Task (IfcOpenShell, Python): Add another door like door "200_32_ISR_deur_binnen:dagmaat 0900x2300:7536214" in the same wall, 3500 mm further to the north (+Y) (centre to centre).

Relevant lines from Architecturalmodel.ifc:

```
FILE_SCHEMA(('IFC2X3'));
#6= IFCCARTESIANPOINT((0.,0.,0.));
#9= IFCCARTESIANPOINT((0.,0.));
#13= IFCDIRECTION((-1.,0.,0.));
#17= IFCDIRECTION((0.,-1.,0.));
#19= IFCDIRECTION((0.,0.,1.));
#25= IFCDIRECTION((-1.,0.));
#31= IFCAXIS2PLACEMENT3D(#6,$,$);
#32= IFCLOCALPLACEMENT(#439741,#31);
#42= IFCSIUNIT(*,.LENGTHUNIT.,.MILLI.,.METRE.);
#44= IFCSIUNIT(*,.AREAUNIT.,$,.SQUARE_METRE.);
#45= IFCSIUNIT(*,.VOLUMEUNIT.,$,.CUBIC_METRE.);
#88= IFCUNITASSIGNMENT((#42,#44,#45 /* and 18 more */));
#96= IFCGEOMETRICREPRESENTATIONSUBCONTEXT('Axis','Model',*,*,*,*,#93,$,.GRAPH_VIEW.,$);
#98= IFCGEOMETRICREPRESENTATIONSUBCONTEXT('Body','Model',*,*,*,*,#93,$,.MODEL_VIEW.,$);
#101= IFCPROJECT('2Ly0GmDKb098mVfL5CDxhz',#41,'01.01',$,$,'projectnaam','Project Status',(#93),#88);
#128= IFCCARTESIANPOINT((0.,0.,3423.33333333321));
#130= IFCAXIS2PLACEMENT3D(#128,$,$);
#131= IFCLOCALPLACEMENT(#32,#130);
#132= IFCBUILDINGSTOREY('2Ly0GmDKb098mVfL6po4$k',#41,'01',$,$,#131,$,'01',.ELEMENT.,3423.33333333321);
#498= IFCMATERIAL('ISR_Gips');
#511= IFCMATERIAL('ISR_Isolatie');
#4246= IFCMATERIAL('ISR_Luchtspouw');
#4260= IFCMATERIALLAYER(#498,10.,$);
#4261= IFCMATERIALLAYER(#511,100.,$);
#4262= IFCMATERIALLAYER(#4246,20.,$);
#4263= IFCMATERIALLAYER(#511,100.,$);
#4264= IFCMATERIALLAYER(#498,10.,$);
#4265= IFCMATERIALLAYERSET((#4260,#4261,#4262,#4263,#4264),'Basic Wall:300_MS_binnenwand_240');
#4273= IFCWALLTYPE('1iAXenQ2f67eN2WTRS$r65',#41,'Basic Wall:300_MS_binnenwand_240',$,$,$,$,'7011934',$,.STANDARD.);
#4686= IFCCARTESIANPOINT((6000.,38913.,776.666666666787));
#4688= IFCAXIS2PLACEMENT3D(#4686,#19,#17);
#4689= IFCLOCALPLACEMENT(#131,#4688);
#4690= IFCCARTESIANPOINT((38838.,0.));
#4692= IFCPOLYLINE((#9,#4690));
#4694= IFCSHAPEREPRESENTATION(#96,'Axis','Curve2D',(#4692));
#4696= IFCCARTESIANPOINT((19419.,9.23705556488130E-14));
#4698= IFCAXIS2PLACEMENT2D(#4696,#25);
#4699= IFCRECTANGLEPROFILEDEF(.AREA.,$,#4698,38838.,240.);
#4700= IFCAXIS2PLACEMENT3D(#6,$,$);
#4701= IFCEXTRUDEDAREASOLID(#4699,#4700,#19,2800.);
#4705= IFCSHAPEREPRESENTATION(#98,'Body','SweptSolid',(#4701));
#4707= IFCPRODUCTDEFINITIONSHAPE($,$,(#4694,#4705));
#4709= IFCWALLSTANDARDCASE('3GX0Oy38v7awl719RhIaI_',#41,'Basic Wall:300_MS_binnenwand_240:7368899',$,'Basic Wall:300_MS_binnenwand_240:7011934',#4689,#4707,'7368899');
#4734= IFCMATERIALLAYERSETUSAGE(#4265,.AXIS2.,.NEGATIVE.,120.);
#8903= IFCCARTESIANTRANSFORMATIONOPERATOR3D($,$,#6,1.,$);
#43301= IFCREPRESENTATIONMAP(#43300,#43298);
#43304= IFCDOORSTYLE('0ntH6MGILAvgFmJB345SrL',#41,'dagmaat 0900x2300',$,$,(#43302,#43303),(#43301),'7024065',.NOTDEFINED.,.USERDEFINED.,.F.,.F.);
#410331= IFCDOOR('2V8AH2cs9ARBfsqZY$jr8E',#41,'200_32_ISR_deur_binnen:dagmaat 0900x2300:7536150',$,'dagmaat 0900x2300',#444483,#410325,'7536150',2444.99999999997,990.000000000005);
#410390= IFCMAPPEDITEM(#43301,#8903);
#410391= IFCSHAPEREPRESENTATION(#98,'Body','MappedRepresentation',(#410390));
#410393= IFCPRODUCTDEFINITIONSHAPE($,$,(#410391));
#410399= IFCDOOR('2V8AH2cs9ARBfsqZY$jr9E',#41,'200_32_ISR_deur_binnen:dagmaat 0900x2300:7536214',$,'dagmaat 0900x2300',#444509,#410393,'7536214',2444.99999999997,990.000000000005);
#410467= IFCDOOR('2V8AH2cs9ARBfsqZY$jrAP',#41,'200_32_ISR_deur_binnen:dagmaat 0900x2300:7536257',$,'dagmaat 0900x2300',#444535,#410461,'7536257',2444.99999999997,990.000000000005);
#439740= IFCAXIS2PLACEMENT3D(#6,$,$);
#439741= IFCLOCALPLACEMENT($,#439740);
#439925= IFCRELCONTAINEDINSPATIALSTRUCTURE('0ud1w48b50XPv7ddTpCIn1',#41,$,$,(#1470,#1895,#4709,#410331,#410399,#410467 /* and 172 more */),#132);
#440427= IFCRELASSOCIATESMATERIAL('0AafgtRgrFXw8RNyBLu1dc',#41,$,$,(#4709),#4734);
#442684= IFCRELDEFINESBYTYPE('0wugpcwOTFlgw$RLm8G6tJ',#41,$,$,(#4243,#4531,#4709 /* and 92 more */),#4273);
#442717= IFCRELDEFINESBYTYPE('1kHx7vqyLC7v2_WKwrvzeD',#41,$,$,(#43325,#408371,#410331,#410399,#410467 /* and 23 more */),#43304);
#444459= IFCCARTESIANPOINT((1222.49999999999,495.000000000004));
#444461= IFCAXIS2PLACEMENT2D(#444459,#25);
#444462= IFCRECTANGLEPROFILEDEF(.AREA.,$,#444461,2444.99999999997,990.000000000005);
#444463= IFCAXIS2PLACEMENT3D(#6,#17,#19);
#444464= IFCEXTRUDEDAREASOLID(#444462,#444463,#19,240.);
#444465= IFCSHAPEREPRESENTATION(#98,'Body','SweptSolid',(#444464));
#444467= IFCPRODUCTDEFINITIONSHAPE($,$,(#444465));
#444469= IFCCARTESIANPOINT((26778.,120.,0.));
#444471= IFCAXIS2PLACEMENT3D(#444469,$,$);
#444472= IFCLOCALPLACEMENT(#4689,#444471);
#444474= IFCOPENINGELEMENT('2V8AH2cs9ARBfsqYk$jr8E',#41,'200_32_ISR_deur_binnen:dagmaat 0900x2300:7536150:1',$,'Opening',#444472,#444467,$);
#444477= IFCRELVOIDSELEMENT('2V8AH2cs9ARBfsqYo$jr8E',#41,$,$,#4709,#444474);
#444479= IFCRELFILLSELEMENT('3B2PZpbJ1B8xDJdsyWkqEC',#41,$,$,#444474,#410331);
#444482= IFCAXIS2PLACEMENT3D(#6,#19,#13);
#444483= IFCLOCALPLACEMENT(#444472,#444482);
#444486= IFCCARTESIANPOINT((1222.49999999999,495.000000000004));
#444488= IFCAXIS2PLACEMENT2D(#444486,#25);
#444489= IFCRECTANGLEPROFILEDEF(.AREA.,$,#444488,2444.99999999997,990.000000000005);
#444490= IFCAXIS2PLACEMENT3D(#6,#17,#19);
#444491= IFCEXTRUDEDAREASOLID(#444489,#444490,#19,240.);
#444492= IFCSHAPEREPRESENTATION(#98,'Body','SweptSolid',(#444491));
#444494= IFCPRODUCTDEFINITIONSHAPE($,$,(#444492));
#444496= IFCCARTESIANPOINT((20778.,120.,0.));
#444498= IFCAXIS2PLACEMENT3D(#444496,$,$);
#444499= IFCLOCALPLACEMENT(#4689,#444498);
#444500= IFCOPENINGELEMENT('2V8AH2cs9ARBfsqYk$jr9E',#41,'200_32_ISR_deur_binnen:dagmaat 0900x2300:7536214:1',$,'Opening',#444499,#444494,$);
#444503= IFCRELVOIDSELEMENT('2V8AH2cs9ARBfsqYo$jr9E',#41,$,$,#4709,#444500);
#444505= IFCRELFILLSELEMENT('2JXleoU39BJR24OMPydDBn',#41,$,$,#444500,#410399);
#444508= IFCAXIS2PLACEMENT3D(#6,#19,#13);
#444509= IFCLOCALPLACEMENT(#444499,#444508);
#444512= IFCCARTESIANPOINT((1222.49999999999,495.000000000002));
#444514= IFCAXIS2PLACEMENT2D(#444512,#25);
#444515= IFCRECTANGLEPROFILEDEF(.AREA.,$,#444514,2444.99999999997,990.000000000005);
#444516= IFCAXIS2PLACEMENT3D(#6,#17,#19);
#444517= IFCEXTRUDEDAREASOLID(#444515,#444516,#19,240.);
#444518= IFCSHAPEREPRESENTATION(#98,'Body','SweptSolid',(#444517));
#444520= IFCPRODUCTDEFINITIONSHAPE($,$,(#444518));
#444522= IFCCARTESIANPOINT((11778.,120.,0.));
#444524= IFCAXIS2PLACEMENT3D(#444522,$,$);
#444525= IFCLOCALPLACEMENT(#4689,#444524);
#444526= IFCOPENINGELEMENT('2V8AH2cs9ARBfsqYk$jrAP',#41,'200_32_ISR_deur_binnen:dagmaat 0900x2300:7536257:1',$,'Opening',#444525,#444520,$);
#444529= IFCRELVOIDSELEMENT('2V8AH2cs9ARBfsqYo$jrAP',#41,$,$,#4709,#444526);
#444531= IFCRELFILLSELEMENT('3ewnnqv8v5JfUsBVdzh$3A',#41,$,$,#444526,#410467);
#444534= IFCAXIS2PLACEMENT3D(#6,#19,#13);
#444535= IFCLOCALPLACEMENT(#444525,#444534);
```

```python
import ifcopenshell
import ifcopenshell.api.feature
import ifcopenshell.api.geometry
import ifcopenshell.api.root
import ifcopenshell.geom
import ifcopenshell.util.element
import ifcopenshell.util.placement
import ifcopenshell.util.shape

model = ifcopenshell.open("Architecturalmodel.ifc")
settings = ifcopenshell.geom.settings()


def volume(element):
    """Net volume in cubic metres, openings subtracted."""
    shape = ifcopenshell.geom.create_shape(settings, element)
    return ifcopenshell.util.shape.get_volume(shape.geometry)


def reuse_history(source, copy):
    """copy_class also copies each property set's owner history, people and application; keep the originals."""
    for rel in copy.IsDefinedBy:
        if rel.is_a("IfcRelDefinesByProperties") and (history := rel.RelatingPropertyDefinition.OwnerHistory):
            rel.RelatingPropertyDefinition.OwnerHistory = source.OwnerHistory
            ifcopenshell.util.element.remove_deep2(model, history)


door = model.by_guid("2V8AH2cs9ARBfsqZY$jr9E")
opening = door.FillsVoids[0].RelatingOpeningElement
wall = opening.VoidsElements[0].RelatingBuildingElement
before = volume(wall)
shift = ifcopenshell.util.placement.get_local_placement(wall.ObjectPlacement)[:3, 0] * -3500.0

# copy_class copies the void relationship, type, container and properties, but no geometry.
new_opening = ifcopenshell.api.root.copy_class(model, product=opening)
new_opening.Representation = ifcopenshell.util.element.copy_deep(
    model, opening.Representation, exclude=["IfcGeometricRepresentationContext", "IfcRepresentationMap"]
)
new_opening.Name = "200_32_ISR_deur_binnen:dagmaat 0900x2300"
new_door = ifcopenshell.api.root.copy_class(model, product=door)
new_door.Representation = ifcopenshell.util.element.copy_deep(
    model, door.Representation, exclude=["IfcGeometricRepresentationContext", "IfcRepresentationMap"]
)
new_door.Name = "200_32_ISR_deur_binnen:dagmaat 0900x2300"
new_door.Tag = None
reuse_history(door, new_door)
fills = ifcopenshell.api.feature.add_filling(model, opening=new_opening, element=new_door)
fills.OwnerHistory = new_door.OwnerHistory  # required in IFC2X3

for old, new in ((opening, new_opening), (door, new_door)):
    matrix = ifcopenshell.util.placement.get_local_placement(old.ObjectPlacement)
    matrix[:3, 3] += shift
    ifcopenshell.api.geometry.edit_object_placement(model, product=new, matrix=matrix, is_si=False)

after = volume(wall)

print(f"wall volume {before:.3f} -> {after:.3f} m3")

model.write("Architecturalmodel_updated.ifc")
```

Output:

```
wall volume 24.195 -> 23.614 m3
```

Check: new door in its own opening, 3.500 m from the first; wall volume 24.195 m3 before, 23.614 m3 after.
